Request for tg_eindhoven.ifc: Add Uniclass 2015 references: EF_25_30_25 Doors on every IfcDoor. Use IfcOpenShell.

First a look at what the model holds.

```python
import ifcopenshell

model = ifcopenshell.open("tg_eindhoven.ifc")
print(model.schema)
print("classifications:", [c.Name for c in model.by_type("IfcClassification")])
for ifc_class in ("IfcDoor", "IfcRoof", "IfcStair", "IfcWall", "IfcWindow"):
    print(ifc_class, len(model.by_type(ifc_class)))
```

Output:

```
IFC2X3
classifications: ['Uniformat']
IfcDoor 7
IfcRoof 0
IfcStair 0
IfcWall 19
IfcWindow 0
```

```python
import ifcopenshell
import ifcopenshell.api.classification

model = ifcopenshell.open("tg_eindhoven.ifc")

# IFC2X3 requires Source and Edition and has no link from the project to the system.
system = model.create_entity("IfcClassification", Source="NBS", Edition="2015", Name="Uniclass 2015")

codes = {
    "IfcDoor": ("EF_25_30_25", "Doors"),
}
for ifc_class, (code, name) in codes.items():
    products = model.by_type(ifc_class)
    ifcopenshell.api.classification.add_reference(
        model, products=products, classification=system, identification=code, name=name
    )
    print(code, len(products))

model.write("tg_eindhoven_rev.ifc")
```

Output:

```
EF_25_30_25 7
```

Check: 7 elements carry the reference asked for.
